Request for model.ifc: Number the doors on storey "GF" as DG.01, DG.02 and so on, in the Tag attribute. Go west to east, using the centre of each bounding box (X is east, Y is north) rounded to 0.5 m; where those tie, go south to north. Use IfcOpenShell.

First a look at what the model holds.

```python
import ifcopenshell
import ifcopenshell.util.element
import ifcopenshell.util.placement

model = ifcopenshell.open("model.ifc")
print(model.schema)
storey = next(s for s in model.by_type("IfcBuildingStorey") if s.Name == "GF")
doors = [e for e in ifcopenshell.util.element.get_decomposition(storey) if e.is_a("IfcDoor")]
for e in sorted(doors, key=lambda e: e.id()):
    origin = ifcopenshell.util.placement.get_local_placement(e.ObjectPlacement)[:3, 3]
    print(e.id(), e.Tag, e.Name, origin.round(2) + 0.0, sep=" | ")
```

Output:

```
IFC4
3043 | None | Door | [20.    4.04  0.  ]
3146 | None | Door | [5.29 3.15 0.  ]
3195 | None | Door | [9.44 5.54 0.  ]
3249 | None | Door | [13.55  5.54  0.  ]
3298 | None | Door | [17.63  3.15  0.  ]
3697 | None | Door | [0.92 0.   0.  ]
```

```python
import ifcopenshell
import ifcopenshell.geom
import ifcopenshell.util.element
import ifcopenshell.util.shape

model = ifcopenshell.open("model.ifc")
settings = ifcopenshell.geom.settings()
settings.set("use-world-coords", True)


def centre(element):
    shape = ifcopenshell.geom.create_shape(settings, element)
    return ifcopenshell.util.shape.get_bbox_centroid(shape.geometry)


storey = next(s for s in model.by_type("IfcBuildingStorey") if s.Name == "GF")
doors = [e for e in ifcopenshell.util.element.get_decomposition(storey) if e.is_a("IfcDoor")]

# Insertion points can sit at a corner or the storey origin, so sort by the geometry (in metres).
centres = {e: centre(e) for e in doors}
doors.sort(key=lambda e: (round(centres[e][0] / 0.5), centres[e][1]))

for i, e in enumerate(doors, start=1):
    number = f"DG.{i:02d}"
    e.Tag = number
    print(e.id(), number)

model.write("model-out.ifc")
```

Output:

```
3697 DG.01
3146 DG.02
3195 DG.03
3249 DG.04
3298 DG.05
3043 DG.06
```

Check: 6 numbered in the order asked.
